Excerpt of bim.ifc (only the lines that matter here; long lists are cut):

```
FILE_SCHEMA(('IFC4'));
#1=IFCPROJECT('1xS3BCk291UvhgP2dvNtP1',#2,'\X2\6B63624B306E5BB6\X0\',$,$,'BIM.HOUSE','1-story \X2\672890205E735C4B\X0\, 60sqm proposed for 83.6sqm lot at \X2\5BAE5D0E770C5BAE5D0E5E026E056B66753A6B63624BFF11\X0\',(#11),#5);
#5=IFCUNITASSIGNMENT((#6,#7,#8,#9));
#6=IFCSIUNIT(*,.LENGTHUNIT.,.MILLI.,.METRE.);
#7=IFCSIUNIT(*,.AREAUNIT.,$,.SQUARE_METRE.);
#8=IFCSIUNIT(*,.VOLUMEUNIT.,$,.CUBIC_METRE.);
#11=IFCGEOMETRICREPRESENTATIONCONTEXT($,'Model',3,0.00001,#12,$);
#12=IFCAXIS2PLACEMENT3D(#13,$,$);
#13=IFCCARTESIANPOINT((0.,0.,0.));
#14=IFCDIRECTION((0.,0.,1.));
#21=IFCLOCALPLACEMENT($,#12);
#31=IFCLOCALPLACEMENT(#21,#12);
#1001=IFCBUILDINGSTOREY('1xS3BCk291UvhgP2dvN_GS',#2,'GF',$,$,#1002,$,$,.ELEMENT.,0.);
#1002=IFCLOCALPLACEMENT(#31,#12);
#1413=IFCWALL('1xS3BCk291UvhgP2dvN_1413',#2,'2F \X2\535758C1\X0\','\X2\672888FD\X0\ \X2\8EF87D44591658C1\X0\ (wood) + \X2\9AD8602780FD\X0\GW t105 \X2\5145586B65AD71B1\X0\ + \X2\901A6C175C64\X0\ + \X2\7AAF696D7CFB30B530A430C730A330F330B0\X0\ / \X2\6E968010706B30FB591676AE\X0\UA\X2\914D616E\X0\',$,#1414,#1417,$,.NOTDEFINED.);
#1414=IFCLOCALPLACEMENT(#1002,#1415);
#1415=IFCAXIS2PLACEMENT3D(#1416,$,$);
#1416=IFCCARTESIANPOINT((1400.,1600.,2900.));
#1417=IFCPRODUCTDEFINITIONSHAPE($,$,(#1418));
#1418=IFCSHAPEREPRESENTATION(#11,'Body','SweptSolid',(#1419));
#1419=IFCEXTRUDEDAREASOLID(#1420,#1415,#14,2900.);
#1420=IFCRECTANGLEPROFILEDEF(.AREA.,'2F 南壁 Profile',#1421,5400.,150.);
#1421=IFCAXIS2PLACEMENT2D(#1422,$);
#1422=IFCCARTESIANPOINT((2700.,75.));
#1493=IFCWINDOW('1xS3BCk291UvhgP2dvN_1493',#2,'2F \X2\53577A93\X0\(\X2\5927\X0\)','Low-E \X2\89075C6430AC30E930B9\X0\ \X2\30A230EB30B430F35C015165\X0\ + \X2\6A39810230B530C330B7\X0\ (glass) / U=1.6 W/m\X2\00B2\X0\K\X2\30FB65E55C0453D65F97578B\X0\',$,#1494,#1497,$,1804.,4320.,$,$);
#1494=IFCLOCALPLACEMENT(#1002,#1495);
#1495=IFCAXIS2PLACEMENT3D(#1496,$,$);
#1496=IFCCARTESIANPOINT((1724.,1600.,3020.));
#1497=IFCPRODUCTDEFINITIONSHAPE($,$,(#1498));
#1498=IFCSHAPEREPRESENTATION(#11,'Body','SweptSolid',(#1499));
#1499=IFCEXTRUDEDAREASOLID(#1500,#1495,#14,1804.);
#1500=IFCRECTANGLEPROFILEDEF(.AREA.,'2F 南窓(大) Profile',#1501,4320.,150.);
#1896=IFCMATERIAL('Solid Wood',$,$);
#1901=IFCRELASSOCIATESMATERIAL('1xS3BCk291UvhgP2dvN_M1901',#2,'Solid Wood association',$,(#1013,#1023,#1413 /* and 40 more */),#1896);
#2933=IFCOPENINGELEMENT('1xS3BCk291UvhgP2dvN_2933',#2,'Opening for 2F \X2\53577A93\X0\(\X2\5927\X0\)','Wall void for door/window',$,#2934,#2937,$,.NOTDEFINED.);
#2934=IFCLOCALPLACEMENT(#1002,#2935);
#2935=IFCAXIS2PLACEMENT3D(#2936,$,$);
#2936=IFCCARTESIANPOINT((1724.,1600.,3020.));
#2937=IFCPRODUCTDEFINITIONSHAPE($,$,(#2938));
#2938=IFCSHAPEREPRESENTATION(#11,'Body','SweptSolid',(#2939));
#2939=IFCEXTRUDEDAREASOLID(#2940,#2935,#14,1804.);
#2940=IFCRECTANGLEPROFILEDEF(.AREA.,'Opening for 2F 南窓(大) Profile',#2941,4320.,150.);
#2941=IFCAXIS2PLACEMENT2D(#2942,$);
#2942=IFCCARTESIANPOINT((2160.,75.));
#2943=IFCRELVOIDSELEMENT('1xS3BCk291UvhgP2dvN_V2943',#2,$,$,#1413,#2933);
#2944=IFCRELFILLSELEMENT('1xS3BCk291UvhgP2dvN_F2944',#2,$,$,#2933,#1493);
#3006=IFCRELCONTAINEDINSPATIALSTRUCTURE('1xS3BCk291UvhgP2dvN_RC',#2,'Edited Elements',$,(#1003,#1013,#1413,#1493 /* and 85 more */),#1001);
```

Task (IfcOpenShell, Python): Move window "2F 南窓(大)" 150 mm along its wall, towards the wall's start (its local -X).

```python
import ifcopenshell
import ifcopenshell.api.geometry
import ifcopenshell.util.placement

model = ifcopenshell.open("bim.ifc")

window = model.by_id(1493)
opening = window.FillsVoids[0].RelatingOpeningElement
wall = opening.VoidsElements[0].RelatingBuildingElement

wall_matrix = ifcopenshell.util.placement.get_local_placement(wall.ObjectPlacement)
shift = wall_matrix[:3, 0] * -150.0
before = ifcopenshell.util.placement.get_local_placement(window.ObjectPlacement)[:3, 3].copy()

# The window is not placed relative to its opening, so move both.
for product in (opening, window):
    matrix = ifcopenshell.util.placement.get_local_placement(product.ObjectPlacement)
    matrix[:3, 3] += shift
    ifcopenshell.api.geometry.edit_object_placement(model, product=product, matrix=matrix, is_si=False)

after = ifcopenshell.util.placement.get_local_placement(window.ObjectPlacement)[:3, 3]
print("window moved by", (after - before).round(3) + 0.0)

model.write("bim-out.ifc")
```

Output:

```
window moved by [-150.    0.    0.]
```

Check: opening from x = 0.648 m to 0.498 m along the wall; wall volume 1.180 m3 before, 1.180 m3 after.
